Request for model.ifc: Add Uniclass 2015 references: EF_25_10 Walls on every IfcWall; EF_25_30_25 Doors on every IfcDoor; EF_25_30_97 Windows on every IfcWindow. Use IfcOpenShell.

First a look at what the model holds.

```python
import ifcopenshell

model = ifcopenshell.open("model.ifc")
print(model.schema)
print("classifications:", [c.Name for c in model.by_type("IfcClassification")])
for ifc_class in ("IfcDoor", "IfcRoof", "IfcStair", "IfcWall", "IfcWindow"):
    print(ifc_class, len(model.by_type(ifc_class)))
```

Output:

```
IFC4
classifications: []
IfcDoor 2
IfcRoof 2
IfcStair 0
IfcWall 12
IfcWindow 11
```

```python
import ifcopenshell
import ifcopenshell.api.classification

model = ifcopenshell.open("model.ifc")

system = ifcopenshell.api.classification.add_classification(model, classification="Uniclass 2015")

codes = {
    "IfcWall": ("EF_25_10", "Walls"),
    "IfcDoor": ("EF_25_30_25", "Doors"),
    "IfcWindow": ("EF_25_30_97", "Windows"),
}
for ifc_class, (code, name) in codes.items():
    products = model.by_type(ifc_class)
    ifcopenshell.api.classification.add_reference(
        model, products=products, classification=system, identification=code, name=name
    )
    print(code, len(products))

model.write("model_rev.ifc")
```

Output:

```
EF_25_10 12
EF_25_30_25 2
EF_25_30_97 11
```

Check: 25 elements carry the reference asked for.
